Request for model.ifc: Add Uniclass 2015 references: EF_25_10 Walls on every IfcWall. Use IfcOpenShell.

First a look at what the model holds.

```python
import ifcopenshell

model = ifcopenshell.open("model.ifc")
print(model.schema)
print("classifications:", [c.Name for c in model.by_type("IfcClassification")])
for ifc_class in ("IfcDoor", "IfcRoof", "IfcStair", "IfcWall", "IfcWindow"):
    print(ifc_class, len(model.by_type(ifc_class)))
```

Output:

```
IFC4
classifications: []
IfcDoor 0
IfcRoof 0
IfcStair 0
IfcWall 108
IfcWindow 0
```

```python
import ifcopenshell
import ifcopenshell.api.classification

model = ifcopenshell.open("model.ifc")

system = ifcopenshell.api.classification.add_classification(model, classification="Uniclass 2015")

codes = {
    "IfcWall": ("EF_25_10", "Walls"),
}
for ifc_class, (code, name) in codes.items():
    products = model.by_type(ifc_class)
    ifcopenshell.api.classification.add_reference(
        model, products=products, classification=system, identification=code, name=name
    )
    print(code, len(products))

model.write("model_rev.ifc")
```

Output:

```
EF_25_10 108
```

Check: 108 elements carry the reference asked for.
